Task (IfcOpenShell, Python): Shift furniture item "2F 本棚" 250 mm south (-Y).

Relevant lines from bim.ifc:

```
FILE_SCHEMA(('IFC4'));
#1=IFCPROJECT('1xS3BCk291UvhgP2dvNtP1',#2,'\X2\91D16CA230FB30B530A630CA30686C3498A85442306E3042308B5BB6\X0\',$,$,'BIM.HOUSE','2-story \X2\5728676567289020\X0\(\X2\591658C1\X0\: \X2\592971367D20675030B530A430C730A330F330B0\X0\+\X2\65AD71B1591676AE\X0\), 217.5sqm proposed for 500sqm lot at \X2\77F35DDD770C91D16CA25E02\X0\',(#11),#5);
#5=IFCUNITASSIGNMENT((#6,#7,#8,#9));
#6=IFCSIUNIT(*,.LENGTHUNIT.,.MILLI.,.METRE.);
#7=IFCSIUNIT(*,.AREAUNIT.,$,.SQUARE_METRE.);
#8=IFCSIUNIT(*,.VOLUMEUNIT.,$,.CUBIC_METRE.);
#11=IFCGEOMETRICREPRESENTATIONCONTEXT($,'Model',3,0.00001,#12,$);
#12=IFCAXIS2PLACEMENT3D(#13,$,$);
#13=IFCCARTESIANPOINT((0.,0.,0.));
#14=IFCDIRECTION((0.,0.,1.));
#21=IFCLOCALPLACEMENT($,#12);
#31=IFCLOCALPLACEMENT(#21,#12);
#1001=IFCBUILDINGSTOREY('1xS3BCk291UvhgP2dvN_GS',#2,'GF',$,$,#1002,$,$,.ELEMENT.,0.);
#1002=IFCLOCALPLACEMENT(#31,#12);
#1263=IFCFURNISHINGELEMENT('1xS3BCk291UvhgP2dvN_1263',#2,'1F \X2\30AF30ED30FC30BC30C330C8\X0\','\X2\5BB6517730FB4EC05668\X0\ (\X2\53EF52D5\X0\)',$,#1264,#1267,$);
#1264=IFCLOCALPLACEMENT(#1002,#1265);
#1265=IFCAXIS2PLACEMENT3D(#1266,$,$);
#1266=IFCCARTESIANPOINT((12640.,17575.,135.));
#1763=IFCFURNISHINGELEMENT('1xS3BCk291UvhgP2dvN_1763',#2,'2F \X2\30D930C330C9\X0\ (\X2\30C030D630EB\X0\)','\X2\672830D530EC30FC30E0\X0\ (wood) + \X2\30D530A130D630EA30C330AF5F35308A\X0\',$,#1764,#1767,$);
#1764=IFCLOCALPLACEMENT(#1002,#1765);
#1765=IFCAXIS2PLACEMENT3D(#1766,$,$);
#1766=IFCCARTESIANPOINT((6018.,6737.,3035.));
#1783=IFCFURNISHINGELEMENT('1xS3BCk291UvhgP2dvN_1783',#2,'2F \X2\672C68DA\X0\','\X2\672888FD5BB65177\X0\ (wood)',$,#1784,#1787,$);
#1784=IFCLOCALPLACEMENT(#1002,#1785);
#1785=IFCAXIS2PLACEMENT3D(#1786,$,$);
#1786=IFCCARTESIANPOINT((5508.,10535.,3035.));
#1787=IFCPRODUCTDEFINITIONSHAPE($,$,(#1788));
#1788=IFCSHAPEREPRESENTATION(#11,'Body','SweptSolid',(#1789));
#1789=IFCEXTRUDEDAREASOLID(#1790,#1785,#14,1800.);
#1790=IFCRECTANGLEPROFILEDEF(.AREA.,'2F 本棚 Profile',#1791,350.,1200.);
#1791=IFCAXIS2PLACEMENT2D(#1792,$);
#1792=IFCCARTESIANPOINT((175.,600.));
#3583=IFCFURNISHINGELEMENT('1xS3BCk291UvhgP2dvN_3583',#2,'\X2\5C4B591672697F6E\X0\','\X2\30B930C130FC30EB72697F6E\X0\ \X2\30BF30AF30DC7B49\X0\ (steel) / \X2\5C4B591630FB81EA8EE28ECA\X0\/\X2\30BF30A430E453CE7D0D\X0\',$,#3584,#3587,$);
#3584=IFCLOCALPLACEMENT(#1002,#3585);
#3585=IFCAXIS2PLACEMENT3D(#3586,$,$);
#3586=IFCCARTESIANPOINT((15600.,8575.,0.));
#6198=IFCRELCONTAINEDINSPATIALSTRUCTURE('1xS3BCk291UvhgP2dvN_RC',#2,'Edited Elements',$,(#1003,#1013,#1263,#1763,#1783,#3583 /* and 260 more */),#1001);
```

```python
import ifcopenshell
import ifcopenshell.api.geometry
import ifcopenshell.util.placement
import ifcopenshell.util.unit

model = ifcopenshell.open("bim.ifc")
unit_scale = ifcopenshell.util.unit.calculate_unit_scale(model)

item = model.by_guid("1xS3BCk291UvhgP2dvN_1783")
matrix = ifcopenshell.util.placement.get_local_placement(item.ObjectPlacement)
matrix[1, 3] -= 0.25 / unit_scale
ifcopenshell.api.geometry.edit_object_placement(model, product=item, matrix=matrix, is_si=False)

print(ifcopenshell.util.placement.get_local_placement(item.ObjectPlacement).round(3) + 0.0)

model.write("bim_rev.ifc")
```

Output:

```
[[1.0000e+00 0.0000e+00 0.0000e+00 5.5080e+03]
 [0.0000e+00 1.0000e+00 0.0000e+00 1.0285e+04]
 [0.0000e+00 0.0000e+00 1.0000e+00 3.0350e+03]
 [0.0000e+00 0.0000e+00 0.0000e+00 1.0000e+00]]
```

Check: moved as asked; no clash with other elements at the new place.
